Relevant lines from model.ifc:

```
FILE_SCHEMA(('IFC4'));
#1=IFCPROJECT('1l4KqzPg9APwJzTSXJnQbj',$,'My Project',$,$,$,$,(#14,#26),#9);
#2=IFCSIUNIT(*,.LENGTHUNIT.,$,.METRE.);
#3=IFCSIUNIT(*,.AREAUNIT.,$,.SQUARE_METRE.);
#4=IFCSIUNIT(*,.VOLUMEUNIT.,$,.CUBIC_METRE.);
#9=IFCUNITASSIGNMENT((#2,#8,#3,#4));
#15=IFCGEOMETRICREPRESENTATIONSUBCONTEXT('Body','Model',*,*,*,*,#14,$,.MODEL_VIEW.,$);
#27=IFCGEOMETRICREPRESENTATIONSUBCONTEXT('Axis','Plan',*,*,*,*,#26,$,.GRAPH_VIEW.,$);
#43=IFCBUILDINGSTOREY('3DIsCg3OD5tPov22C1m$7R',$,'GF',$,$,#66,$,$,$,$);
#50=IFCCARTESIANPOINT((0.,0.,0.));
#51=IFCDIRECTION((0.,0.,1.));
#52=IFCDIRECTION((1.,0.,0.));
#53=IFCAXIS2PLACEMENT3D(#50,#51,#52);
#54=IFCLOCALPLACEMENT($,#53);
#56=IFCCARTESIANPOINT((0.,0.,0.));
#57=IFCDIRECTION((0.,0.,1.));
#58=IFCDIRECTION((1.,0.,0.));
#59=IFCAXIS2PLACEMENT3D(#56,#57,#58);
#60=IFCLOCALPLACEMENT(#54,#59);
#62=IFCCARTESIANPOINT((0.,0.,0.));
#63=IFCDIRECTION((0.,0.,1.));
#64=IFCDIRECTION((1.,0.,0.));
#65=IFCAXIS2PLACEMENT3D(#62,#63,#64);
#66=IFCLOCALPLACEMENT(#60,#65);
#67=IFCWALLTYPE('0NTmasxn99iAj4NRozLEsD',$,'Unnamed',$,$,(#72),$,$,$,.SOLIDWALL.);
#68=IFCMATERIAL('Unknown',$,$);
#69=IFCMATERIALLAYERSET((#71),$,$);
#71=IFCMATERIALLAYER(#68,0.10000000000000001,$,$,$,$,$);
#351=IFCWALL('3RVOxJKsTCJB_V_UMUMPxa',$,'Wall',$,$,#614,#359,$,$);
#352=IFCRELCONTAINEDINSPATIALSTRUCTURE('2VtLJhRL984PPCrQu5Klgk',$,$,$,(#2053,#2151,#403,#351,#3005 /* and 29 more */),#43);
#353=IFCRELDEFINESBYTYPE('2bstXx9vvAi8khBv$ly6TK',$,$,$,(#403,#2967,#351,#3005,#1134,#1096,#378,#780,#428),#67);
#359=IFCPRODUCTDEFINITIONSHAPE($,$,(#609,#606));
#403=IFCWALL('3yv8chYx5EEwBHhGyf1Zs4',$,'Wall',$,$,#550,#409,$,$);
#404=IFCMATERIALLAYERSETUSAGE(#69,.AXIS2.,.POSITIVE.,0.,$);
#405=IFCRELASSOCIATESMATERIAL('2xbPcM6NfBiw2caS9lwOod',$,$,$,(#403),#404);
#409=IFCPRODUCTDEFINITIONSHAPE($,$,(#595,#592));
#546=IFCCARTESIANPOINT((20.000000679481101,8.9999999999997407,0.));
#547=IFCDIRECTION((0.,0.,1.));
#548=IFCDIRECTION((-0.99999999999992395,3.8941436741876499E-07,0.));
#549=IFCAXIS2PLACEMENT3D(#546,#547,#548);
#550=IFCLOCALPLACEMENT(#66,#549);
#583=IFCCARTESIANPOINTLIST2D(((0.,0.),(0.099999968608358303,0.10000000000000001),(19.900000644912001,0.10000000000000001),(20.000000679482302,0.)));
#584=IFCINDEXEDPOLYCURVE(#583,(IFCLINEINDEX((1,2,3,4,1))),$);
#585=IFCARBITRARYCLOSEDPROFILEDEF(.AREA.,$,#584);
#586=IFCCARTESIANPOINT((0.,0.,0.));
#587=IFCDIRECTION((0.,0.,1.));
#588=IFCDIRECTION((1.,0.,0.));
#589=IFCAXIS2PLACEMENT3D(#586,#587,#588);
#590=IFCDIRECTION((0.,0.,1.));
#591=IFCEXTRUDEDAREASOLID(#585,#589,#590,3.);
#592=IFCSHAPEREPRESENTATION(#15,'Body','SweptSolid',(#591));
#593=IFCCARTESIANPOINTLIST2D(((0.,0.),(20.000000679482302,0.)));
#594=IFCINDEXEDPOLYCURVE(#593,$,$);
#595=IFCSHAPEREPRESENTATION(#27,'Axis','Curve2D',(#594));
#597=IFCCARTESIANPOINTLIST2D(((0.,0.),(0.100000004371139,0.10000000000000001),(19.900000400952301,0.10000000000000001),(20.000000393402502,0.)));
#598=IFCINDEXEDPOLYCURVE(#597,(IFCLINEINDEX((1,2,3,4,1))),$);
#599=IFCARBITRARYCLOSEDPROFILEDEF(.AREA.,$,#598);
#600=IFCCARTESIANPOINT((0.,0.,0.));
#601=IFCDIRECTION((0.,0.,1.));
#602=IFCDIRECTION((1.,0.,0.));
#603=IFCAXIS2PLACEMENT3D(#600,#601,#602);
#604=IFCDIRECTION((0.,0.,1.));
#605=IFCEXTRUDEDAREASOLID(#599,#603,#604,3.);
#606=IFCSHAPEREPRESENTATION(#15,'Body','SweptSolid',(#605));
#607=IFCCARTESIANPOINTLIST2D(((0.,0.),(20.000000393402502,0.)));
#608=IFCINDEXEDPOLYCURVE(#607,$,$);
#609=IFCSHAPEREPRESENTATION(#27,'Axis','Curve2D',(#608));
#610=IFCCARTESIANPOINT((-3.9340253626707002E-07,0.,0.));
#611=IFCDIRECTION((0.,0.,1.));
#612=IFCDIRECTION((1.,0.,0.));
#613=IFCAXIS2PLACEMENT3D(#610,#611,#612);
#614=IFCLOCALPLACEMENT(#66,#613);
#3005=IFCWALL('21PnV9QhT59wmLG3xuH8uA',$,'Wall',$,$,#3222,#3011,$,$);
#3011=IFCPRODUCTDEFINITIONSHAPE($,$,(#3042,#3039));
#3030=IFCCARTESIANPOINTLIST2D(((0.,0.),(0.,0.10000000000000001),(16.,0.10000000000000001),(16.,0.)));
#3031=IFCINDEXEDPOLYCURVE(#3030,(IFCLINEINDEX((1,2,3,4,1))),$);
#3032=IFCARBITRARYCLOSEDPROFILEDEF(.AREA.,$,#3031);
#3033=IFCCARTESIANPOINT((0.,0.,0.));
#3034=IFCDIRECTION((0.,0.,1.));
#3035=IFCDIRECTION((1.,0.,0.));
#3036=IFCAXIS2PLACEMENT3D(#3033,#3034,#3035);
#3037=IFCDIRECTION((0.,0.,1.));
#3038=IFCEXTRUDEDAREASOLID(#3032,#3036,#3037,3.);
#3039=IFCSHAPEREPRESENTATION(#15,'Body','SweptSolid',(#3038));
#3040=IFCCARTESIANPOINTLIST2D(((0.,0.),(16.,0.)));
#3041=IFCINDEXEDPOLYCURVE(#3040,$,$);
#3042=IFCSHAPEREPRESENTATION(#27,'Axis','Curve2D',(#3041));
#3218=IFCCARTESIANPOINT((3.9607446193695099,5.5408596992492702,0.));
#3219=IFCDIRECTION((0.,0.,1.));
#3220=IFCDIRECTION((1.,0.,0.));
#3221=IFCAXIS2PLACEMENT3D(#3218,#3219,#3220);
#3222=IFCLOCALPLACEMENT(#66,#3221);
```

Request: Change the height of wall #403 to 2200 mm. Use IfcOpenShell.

```python
import ifcopenshell
import ifcopenshell.geom
import ifcopenshell.util.representation
import ifcopenshell.util.shape

model = ifcopenshell.open("model.ifc")
settings = ifcopenshell.geom.settings()


def volume(element):
    """Net volume in cubic metres, openings subtracted."""
    shape = ifcopenshell.geom.create_shape(settings, element)
    return ifcopenshell.util.shape.get_volume(shape.geometry)


wall = model.by_id(403)
before = volume(wall)

body = ifcopenshell.util.representation.get_representation(wall, "Model", "Body")
solid = body.Items[0]
old_height = solid.Depth
solid.Depth = 2.2
after = volume(wall)

print(f"height {old_height:g} -> {solid.Depth:g}, volume {before:.3f} -> {after:.3f} m3")

model.write("model-out.ifc")
```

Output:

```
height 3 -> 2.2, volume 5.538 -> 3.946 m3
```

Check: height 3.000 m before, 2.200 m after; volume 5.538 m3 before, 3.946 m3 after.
